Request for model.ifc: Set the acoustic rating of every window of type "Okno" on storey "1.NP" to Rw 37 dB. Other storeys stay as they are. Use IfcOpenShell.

First a look at what the model holds.

```python
import ifcopenshell
import ifcopenshell.util.element

model = ifcopenshell.open("model.ifc")
print(model.schema)
storey = next(s for s in model.by_type("IfcBuildingStorey") if s.Name == "1.NP")
windows = [e for e in ifcopenshell.util.element.get_decomposition(storey) if e.is_a("IfcWindow")]
seen = {}
for e in windows:
    element_type = ifcopenshell.util.element.get_type(e)
    key = (element_type.Name if element_type != e and element_type else None, ifcopenshell.util.element.get_pset(e, "Pset_WindowCommon", "AcousticRating"))
    seen[key] = seen.get(key, 0) + 1
for (name, value), count in sorted(seen.items(), key=str):
    print(count, "x", name, "|", value)
```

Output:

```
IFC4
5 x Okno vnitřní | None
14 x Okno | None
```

```python
import ifcopenshell
import ifcopenshell.api.pset
import ifcopenshell.util.element

model = ifcopenshell.open("model.ifc")

storey = next(s for s in model.by_type("IfcBuildingStorey") if s.Name == "1.NP")
windows = [e for e in ifcopenshell.util.element.get_decomposition(storey) if e.is_a("IfcWindow")]

count = 0
for e in windows:
    element_type = ifcopenshell.util.element.get_type(e)
    if element_type in (None, e) or element_type.Name != "Okno":
        continue
    # add_pset returns the element's existing set when there is one.
    pset = ifcopenshell.api.pset.add_pset(model, product=e, name="Pset_WindowCommon")
    ifcopenshell.api.pset.edit_pset(model, pset=pset, properties={"AcousticRating": "Rw 37 dB"})
    count += 1

print(count, "windows updated")

model.write("model_rev.ifc")
```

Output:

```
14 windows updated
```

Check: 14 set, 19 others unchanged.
